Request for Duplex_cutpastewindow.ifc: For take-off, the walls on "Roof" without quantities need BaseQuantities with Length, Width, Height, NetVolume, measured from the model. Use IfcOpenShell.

First a look at what the model holds.

```python
import ifcopenshell
import ifcopenshell.util.element
import ifcopenshell.util.unit

model = ifcopenshell.open("Duplex_cutpastewindow.ifc")
print(model.schema)
for unit_type in ("LENGTHUNIT", "AREAUNIT", "VOLUMEUNIT"):
    print(unit_type, ifcopenshell.util.unit.calculate_unit_scale(model, unit_type))
storey = next(s for s in model.by_type("IfcBuildingStorey") if s.Name == "Roof")
walls = [e for e in ifcopenshell.util.element.get_decomposition(storey) if e.is_a("IfcWall")]
for e in sorted(walls, key=lambda e: e.id()):
    print(e.id(), e.is_a(), e.Name, list(ifcopenshell.util.element.get_psets(e, qtos_only=True)), sep=" | ")
```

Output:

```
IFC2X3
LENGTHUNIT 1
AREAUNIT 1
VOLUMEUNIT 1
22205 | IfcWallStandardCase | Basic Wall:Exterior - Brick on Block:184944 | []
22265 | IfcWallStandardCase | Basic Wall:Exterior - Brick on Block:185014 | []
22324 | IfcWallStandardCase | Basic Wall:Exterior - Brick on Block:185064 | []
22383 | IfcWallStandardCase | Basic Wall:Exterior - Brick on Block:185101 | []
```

```python
import ifcopenshell
import ifcopenshell.api.pset
import ifcopenshell.geom
import ifcopenshell.util.element
import ifcopenshell.util.shape
import ifcopenshell.util.unit

model = ifcopenshell.open("Duplex_cutpastewindow.ifc")
unit_scale = ifcopenshell.util.unit.calculate_unit_scale(model)
volume_scale = ifcopenshell.util.unit.calculate_unit_scale(model, "VOLUMEUNIT")
settings = ifcopenshell.geom.settings()

storey = next(s for s in model.by_type("IfcBuildingStorey") if s.Name == "Roof")
walls = [e for e in ifcopenshell.util.element.get_decomposition(storey) if e.is_a("IfcWall")]

for e in sorted(walls, key=lambda e: e.id()):
    if ifcopenshell.util.element.get_psets(e, qtos_only=True, should_inherit=False):
        continue
    # Geometry comes back in metres, in the element's own axes.
    shape = ifcopenshell.geom.create_shape(settings, e)
    values = {
        "Length": ifcopenshell.util.shape.get_x(shape.geometry) / unit_scale,
        "Width": ifcopenshell.util.shape.get_y(shape.geometry) / unit_scale,
        "Height": ifcopenshell.util.shape.get_z(shape.geometry) / unit_scale,
        "NetVolume": ifcopenshell.util.shape.get_volume(shape.geometry) / volume_scale,
    }
    qto = ifcopenshell.api.pset.add_qto(model, product=e, name="BaseQuantities")
    ifcopenshell.api.pset.edit_qto(model, qto=qto, properties=values)
    print(e.id(), {k: round(v, 3) for k, v in values.items()})

model.write("Duplex_cutpastewindow_v2.ifc")
```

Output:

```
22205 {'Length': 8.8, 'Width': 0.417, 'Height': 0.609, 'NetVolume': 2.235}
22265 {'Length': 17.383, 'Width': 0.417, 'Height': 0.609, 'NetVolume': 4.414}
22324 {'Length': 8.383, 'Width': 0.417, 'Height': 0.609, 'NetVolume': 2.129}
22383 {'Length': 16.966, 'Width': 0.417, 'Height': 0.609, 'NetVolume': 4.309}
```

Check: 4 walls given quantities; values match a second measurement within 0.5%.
